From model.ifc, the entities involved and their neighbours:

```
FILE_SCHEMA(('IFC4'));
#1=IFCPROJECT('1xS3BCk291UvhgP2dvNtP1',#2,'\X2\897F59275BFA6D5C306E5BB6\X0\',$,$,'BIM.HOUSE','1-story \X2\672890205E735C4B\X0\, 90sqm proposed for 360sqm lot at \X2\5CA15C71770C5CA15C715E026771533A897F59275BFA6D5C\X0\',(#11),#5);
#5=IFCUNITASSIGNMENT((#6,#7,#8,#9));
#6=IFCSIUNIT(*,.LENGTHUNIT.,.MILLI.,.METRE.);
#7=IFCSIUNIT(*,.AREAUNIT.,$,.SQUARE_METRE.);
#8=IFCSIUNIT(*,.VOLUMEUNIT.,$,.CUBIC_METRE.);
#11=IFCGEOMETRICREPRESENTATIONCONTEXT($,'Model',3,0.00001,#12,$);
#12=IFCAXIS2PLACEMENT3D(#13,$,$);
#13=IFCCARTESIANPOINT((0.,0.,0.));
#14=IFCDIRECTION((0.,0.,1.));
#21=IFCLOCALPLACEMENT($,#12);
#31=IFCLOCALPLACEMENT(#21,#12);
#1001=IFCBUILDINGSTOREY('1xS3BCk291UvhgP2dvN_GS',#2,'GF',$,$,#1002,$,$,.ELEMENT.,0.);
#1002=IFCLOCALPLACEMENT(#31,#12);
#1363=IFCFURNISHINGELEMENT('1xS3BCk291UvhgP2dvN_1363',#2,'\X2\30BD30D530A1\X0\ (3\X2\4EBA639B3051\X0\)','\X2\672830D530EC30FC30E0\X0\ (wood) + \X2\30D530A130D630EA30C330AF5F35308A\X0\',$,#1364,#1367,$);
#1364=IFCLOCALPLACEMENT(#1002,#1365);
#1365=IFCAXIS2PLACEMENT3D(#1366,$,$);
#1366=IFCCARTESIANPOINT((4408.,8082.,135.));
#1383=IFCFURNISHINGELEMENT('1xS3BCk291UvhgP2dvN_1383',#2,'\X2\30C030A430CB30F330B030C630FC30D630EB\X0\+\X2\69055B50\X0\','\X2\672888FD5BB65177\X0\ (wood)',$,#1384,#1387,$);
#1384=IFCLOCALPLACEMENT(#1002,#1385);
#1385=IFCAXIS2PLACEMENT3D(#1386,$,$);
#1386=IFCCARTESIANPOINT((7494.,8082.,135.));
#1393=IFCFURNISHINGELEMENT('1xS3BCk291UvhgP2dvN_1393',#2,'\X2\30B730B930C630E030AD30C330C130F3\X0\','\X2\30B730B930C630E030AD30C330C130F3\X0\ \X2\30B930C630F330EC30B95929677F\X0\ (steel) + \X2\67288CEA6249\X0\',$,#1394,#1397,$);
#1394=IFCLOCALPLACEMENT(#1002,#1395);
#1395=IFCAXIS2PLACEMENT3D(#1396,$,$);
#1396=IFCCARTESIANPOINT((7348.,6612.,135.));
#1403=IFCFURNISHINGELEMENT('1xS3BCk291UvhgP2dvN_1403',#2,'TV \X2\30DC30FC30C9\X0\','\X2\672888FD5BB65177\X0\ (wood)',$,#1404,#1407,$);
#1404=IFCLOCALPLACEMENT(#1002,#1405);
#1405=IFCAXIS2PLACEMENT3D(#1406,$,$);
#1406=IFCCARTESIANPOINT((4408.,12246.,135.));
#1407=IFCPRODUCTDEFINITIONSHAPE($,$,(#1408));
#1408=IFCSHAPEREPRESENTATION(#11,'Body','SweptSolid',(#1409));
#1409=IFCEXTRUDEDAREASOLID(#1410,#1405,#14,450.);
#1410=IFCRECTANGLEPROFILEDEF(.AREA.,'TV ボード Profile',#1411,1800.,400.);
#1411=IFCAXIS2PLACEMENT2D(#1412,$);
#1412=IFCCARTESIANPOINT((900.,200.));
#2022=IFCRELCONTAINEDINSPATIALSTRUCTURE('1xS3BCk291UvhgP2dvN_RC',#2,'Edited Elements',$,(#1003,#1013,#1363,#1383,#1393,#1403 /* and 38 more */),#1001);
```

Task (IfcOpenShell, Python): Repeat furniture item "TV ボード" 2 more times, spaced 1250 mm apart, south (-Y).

```python
import numpy as np
import ifcopenshell
import ifcopenshell.api.geometry
import ifcopenshell.api.root
import ifcopenshell.util.element
import ifcopenshell.util.placement
import ifcopenshell.util.unit

model = ifcopenshell.open("model.ifc")
unit_scale = ifcopenshell.util.unit.calculate_unit_scale(model)


def reuse_history(source, copy):
    """copy_class also copies each property set's owner history, people and application; keep the originals."""
    for rel in copy.IsDefinedBy:
        if rel.is_a("IfcRelDefinesByProperties") and (history := rel.RelatingPropertyDefinition.OwnerHistory):
            rel.RelatingPropertyDefinition.OwnerHistory = source.OwnerHistory
            ifcopenshell.util.element.remove_deep2(model, history)


source = model.by_id(1403)
base = ifcopenshell.util.placement.get_local_placement(source.ObjectPlacement)
step = np.array([0.0, -1.0, 0.0]) * 1.25 / unit_scale

for i in range(1, 3):
    copy = ifcopenshell.api.root.copy_class(model, product=source)
    copy.Representation = ifcopenshell.util.element.copy_deep(
        model, source.Representation, exclude=["IfcGeometricRepresentationContext", "IfcRepresentationMap"]
    )
    reuse_history(source, copy)
    matrix = base.copy()
    matrix[:3, 3] += i * step
    print("added at", matrix[:3, 3].round(3) + 0.0)
    ifcopenshell.api.geometry.edit_object_placement(model, product=copy, matrix=matrix, is_si=False)

model.write("model_updated.ifc")
```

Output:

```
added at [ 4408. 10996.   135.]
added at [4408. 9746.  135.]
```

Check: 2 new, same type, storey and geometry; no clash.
